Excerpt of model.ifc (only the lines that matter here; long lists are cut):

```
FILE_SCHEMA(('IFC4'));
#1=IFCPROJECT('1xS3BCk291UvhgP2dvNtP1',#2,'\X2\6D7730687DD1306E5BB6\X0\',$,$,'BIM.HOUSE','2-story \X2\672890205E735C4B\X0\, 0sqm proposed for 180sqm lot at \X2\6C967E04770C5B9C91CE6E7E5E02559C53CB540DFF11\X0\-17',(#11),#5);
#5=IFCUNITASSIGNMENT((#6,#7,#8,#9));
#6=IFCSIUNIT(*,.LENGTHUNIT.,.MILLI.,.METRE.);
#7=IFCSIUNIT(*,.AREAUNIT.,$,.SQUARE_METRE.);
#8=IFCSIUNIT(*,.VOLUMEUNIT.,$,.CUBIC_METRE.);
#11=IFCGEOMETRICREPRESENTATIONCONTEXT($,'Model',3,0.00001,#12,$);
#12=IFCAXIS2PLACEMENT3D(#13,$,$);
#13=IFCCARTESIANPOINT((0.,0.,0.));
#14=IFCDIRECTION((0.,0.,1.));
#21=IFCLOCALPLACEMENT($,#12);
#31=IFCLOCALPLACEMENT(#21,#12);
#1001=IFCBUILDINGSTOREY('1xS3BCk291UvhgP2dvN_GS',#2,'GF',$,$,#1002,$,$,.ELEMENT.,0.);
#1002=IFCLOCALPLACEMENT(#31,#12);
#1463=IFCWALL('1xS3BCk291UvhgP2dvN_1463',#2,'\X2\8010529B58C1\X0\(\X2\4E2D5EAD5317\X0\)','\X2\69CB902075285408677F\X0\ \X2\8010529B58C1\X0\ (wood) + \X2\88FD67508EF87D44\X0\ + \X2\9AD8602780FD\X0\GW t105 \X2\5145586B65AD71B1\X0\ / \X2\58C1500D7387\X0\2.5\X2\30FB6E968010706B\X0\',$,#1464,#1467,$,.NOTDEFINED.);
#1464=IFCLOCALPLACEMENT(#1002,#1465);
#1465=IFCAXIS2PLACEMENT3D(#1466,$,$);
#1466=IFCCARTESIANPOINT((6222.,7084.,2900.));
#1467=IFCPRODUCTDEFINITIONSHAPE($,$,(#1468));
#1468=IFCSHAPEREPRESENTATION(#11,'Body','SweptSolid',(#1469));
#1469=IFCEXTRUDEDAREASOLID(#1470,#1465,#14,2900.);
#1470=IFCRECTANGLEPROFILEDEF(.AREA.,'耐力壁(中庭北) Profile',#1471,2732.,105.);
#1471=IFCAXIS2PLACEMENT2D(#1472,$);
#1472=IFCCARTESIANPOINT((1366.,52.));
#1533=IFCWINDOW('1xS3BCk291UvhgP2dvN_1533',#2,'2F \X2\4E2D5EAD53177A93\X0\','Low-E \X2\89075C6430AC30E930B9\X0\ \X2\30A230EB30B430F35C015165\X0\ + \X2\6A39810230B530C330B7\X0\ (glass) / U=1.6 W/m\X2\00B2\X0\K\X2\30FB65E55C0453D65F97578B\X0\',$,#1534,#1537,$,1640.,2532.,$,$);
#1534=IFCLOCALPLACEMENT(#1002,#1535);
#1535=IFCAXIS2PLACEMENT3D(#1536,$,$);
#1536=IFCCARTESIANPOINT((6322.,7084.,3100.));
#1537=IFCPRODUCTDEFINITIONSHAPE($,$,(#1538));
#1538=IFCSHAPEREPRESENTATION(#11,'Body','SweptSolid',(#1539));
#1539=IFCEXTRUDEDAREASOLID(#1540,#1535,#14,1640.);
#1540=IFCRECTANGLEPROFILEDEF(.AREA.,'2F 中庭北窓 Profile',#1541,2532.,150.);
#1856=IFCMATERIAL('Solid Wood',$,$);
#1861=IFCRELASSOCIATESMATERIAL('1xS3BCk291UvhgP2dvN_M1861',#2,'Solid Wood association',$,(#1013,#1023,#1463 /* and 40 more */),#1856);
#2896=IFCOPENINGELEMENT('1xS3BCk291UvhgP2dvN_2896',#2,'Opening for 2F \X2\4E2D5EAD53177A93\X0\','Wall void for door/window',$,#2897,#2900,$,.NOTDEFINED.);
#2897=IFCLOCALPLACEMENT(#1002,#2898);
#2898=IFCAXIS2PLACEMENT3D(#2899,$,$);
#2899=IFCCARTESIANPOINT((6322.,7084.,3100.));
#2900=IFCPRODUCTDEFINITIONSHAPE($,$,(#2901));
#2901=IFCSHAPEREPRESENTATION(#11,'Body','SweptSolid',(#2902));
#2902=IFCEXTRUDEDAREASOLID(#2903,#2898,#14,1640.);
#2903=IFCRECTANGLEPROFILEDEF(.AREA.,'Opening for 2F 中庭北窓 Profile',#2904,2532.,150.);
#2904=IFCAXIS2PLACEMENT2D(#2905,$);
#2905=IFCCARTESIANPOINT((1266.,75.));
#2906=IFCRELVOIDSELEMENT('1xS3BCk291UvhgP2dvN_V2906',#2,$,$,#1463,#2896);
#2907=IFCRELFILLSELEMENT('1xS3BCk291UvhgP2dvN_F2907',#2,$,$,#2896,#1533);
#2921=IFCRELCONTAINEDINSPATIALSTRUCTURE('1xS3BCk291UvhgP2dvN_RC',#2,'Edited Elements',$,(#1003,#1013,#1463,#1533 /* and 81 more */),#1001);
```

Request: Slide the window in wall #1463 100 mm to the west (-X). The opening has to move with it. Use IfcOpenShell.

```python
import ifcopenshell
import ifcopenshell.api.geometry
import ifcopenshell.util.placement

model = ifcopenshell.open("model.ifc")

window = model.by_guid("1xS3BCk291UvhgP2dvN_1533")
opening = window.FillsVoids[0].RelatingOpeningElement
wall = opening.VoidsElements[0].RelatingBuildingElement

wall_matrix = ifcopenshell.util.placement.get_local_placement(wall.ObjectPlacement)
shift = wall_matrix[:3, 0] * -100.0
before = ifcopenshell.util.placement.get_local_placement(window.ObjectPlacement)[:3, 3].copy()

# The window is not placed relative to its opening, so move both.
for product in (opening, window):
    matrix = ifcopenshell.util.placement.get_local_placement(product.ObjectPlacement)
    matrix[:3, 3] += shift
    ifcopenshell.api.geometry.edit_object_placement(model, product=product, matrix=matrix, is_si=False)

after = ifcopenshell.util.placement.get_local_placement(window.ObjectPlacement)[:3, 3]
print("window moved by", (after - before).round(3) + 0.0)

model.write("model_edited.ifc")
```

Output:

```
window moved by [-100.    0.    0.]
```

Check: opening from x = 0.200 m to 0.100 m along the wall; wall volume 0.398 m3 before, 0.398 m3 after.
